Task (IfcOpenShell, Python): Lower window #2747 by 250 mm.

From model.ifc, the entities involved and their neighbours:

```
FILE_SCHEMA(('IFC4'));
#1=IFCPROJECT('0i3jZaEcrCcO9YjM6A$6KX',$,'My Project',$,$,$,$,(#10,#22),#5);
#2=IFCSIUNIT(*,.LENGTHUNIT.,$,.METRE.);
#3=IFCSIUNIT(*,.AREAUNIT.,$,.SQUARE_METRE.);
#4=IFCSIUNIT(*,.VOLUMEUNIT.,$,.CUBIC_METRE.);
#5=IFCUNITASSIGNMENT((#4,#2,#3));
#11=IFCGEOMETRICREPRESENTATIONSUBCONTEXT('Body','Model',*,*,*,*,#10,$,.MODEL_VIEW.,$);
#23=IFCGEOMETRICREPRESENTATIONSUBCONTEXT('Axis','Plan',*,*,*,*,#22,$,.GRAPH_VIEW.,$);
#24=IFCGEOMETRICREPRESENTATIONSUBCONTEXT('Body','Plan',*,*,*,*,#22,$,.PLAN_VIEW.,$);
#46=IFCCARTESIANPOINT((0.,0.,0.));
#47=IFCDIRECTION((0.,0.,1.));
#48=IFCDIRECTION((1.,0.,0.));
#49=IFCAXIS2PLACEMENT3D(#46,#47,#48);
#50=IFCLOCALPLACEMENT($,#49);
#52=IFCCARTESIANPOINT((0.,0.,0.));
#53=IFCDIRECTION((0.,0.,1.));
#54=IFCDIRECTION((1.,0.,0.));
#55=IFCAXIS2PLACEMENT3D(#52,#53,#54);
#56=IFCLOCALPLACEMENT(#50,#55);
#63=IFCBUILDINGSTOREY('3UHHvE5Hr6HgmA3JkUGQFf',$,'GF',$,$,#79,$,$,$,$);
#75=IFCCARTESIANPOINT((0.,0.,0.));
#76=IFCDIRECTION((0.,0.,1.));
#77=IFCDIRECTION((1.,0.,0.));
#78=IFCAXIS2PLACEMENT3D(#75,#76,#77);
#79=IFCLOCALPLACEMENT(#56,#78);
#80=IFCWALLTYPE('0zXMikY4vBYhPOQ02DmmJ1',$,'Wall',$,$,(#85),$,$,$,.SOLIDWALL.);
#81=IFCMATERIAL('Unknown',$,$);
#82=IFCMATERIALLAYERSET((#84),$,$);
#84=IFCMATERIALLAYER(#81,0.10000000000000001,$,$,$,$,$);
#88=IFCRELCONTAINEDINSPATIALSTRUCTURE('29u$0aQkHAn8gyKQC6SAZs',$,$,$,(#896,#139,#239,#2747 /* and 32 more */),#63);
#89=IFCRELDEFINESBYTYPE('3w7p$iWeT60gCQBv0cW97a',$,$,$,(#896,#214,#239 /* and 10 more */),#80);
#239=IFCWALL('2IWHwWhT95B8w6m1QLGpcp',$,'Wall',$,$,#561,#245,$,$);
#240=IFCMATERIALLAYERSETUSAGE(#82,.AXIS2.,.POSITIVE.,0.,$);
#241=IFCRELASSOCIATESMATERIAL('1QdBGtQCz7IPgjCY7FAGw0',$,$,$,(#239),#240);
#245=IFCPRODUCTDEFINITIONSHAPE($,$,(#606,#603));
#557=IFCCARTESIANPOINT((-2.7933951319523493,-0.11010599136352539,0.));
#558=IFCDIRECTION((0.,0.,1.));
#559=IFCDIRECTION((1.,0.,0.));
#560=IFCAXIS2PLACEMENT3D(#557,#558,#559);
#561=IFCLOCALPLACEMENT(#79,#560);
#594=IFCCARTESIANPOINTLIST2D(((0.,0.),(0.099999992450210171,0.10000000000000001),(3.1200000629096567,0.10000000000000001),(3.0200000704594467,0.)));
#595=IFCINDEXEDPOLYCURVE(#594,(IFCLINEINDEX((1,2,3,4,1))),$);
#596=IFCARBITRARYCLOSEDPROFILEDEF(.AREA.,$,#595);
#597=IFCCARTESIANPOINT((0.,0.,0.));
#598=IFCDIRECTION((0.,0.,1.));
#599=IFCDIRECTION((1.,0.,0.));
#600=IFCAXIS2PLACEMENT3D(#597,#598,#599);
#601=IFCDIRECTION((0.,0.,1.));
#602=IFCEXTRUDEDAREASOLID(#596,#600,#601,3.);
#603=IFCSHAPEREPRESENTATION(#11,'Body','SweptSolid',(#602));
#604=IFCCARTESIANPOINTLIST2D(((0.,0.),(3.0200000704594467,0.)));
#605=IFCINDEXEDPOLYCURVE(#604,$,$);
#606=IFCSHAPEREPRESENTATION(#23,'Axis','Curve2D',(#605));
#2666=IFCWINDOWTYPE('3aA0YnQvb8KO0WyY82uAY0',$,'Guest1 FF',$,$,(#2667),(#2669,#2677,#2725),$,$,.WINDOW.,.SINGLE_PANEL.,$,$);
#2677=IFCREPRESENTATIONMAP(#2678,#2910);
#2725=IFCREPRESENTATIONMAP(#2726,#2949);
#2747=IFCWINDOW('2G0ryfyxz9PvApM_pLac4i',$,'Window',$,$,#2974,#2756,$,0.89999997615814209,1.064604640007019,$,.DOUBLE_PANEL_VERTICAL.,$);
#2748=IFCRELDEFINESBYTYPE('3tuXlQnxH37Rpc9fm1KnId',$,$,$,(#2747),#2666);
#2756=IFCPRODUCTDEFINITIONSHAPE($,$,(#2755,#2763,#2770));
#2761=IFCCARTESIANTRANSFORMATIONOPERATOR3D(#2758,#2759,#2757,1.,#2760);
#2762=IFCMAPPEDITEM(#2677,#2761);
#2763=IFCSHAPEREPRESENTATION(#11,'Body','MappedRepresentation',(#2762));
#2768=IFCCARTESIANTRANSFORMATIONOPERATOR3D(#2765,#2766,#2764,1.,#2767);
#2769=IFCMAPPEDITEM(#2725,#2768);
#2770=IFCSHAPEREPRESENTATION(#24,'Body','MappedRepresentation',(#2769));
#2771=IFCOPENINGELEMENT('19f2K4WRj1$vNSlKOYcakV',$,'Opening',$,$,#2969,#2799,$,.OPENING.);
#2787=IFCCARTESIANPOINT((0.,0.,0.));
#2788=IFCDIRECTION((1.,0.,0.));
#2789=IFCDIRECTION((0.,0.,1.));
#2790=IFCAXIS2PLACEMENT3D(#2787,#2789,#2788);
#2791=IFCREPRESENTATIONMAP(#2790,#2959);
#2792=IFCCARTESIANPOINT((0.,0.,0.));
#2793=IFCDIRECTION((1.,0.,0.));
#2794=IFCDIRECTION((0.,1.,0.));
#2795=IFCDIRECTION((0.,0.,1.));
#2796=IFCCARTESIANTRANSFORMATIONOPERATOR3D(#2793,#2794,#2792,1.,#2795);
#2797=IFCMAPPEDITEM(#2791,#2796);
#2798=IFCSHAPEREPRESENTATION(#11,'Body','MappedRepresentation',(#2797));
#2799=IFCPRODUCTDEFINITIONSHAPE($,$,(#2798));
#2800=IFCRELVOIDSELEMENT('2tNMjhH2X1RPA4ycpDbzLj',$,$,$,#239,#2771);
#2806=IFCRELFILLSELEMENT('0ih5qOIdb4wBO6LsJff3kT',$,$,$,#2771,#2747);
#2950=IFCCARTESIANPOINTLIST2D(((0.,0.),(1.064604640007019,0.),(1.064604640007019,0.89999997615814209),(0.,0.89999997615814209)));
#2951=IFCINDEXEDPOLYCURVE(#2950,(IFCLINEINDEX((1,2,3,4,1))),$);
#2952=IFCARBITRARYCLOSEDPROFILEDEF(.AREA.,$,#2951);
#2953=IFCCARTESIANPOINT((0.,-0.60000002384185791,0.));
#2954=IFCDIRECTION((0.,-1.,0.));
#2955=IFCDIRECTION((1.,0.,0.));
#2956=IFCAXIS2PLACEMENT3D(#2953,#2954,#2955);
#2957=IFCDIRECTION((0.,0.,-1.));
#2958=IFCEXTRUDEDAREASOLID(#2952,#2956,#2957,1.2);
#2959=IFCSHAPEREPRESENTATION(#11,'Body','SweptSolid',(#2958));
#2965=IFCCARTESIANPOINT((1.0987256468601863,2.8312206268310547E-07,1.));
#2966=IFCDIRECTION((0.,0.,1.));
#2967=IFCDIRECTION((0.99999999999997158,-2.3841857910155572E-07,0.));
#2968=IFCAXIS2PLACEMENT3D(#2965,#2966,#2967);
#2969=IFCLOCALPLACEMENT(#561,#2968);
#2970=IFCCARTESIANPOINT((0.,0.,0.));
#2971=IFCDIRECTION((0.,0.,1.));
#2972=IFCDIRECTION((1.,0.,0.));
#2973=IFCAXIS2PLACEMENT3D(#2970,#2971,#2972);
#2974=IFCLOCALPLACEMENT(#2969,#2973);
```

```python
import numpy as np
import ifcopenshell
import ifcopenshell.api.geometry
import ifcopenshell.util.placement
import ifcopenshell.util.unit

model = ifcopenshell.open("model.ifc")
unit_scale = ifcopenshell.util.unit.calculate_unit_scale(model)

window = model.by_guid("2G0ryfyxz9PvApM_pLac4i")
opening = window.FillsVoids[0].RelatingOpeningElement
dz = -0.25

shift = np.array([0.0, 0.0, dz])
# The window is placed relative to its opening, so it follows when the opening moves.
matrix = ifcopenshell.util.placement.get_local_placement(opening.ObjectPlacement)
matrix[:3, 3] += shift
ifcopenshell.api.geometry.edit_object_placement(
    model, product=opening, matrix=matrix, is_si=False, should_transform_children=True
)

print(f"moved by {dz * unit_scale:+.3f} m")

model.write("model_rev.ifc")
```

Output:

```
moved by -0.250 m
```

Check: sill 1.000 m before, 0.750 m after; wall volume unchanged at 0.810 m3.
